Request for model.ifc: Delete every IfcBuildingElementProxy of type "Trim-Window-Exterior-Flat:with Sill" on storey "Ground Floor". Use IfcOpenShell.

First a look at what the model holds.

```python
import ifcopenshell
import ifcopenshell.util.element

model = ifcopenshell.open("model.ifc")
print(model.schema)
storey = next(s for s in model.by_type("IfcBuildingStorey") if s.Name == "Ground Floor")
proxies = [e for e in ifcopenshell.util.element.get_decomposition(storey) if e.is_a("IfcBuildingElementProxy")]
seen = {}
for e in proxies:
    element_type = ifcopenshell.util.element.get_type(e)
    name = element_type.Name if element_type not in (None, e) else None
    seen[name] = seen.get(name, 0) + 1
for name, count in sorted(seen.items(), key=str):
    print(count, "x", name)
```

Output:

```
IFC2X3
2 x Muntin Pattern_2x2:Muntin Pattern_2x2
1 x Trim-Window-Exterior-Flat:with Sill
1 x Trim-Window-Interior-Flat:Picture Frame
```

```python
import ifcopenshell
import ifcopenshell.api.root
import ifcopenshell.util.element

model = ifcopenshell.open("model.ifc")

storey = next(s for s in model.by_type("IfcBuildingStorey") if s.Name == "Ground Floor")
proxies = [e for e in ifcopenshell.util.element.get_decomposition(storey) if e.is_a("IfcBuildingElementProxy")]
targets = [e for e in proxies if (t := ifcopenshell.util.element.get_type(e)) not in (None, e) and t.Name == "Trim-Window-Exterior-Flat:with Sill"]

for e in targets:
    ifcopenshell.api.root.remove_product(model, product=e)
print(len(targets), "removed")

model.write("model_edited.ifc")
```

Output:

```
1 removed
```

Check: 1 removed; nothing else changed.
